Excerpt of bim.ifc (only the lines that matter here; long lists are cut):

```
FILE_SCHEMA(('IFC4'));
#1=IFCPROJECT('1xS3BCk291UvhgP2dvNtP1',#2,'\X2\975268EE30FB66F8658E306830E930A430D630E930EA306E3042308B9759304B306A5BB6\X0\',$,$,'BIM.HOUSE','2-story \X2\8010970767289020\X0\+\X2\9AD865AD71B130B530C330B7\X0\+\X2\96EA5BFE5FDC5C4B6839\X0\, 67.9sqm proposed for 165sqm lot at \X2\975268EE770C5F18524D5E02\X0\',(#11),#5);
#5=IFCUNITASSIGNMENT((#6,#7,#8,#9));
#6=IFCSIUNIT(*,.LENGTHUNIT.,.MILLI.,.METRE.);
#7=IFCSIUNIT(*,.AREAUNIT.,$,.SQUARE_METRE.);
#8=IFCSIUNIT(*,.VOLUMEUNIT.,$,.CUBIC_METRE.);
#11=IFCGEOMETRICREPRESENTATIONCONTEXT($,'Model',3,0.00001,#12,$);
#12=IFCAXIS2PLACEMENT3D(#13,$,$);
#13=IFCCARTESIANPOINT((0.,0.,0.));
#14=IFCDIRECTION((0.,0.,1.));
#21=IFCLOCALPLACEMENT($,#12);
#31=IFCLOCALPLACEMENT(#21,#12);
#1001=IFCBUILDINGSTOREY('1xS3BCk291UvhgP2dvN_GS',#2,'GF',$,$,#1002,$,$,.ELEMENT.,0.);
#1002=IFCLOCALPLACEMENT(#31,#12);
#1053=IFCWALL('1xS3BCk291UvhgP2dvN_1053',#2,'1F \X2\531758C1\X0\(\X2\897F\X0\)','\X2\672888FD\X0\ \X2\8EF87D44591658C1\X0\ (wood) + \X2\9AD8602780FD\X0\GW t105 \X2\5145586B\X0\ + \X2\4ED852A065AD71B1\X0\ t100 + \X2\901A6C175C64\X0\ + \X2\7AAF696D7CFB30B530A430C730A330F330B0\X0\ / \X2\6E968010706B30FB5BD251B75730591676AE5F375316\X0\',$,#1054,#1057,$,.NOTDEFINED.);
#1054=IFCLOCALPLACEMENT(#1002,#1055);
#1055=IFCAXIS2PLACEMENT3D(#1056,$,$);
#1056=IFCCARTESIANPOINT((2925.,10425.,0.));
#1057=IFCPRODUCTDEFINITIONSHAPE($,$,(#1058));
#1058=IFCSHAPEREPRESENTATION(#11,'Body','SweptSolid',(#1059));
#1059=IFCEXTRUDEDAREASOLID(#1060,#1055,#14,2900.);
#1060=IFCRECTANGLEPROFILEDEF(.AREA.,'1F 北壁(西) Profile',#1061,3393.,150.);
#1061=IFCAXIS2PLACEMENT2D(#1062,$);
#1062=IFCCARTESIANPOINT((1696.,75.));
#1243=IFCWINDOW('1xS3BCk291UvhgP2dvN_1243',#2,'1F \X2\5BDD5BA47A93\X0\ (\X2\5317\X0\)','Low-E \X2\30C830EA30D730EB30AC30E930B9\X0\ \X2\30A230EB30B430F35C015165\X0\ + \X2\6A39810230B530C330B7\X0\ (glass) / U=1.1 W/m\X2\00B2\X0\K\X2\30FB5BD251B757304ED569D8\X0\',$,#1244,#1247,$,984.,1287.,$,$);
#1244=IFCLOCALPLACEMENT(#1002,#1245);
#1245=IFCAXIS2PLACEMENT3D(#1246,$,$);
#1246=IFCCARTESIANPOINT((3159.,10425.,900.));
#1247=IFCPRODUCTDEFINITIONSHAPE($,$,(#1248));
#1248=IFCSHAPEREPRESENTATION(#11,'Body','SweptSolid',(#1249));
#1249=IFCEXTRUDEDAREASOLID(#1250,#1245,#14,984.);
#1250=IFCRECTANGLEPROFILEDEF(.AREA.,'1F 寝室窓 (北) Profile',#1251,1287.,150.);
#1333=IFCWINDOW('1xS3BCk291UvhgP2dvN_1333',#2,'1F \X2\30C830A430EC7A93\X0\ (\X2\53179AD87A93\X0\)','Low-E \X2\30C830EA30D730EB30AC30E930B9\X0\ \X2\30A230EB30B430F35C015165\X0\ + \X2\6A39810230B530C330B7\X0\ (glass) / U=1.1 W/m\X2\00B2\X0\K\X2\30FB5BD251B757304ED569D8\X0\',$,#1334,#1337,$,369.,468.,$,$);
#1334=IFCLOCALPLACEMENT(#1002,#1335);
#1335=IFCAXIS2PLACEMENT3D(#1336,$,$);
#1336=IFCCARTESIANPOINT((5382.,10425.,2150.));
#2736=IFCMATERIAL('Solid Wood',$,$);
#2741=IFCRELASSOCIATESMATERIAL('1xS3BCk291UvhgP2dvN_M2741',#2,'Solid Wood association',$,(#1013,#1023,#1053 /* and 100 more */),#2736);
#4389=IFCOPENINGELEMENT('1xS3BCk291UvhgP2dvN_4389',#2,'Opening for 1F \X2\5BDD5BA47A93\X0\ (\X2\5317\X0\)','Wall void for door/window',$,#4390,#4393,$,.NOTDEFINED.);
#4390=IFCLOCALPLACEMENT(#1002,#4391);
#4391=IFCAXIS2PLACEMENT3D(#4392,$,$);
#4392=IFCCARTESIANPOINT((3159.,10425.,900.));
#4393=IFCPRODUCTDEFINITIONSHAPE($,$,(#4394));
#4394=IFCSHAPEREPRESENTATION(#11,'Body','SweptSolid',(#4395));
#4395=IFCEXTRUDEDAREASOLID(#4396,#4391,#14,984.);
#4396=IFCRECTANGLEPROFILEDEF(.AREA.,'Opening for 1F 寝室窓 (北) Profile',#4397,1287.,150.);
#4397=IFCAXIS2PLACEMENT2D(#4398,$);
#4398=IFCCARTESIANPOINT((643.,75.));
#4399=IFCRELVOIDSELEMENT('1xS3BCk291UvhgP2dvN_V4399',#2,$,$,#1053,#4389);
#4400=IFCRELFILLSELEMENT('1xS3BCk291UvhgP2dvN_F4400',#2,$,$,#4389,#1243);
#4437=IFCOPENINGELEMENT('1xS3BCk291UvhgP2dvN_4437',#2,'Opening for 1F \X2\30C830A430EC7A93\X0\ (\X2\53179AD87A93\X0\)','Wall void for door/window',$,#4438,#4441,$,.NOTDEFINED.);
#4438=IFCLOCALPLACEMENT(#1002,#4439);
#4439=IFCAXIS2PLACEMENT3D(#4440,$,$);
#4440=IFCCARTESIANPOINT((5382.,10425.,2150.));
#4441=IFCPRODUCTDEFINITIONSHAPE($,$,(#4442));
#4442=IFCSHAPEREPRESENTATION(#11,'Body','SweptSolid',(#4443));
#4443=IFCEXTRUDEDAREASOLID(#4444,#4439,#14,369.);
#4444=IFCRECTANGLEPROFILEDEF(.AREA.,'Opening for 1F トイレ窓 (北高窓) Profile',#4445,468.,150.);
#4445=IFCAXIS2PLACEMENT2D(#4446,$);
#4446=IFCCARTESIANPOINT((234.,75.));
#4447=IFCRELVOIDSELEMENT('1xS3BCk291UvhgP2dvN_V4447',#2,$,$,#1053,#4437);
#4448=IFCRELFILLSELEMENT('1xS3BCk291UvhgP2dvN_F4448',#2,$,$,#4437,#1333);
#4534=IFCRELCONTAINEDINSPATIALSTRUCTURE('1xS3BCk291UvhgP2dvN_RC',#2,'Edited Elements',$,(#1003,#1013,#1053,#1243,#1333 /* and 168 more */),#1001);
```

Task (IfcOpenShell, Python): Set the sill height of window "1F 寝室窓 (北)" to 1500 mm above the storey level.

```python
import numpy as np
import ifcopenshell
import ifcopenshell.api.geometry
import ifcopenshell.geom
import ifcopenshell.util.element
import ifcopenshell.util.placement
import ifcopenshell.util.shape
import ifcopenshell.util.unit

model = ifcopenshell.open("bim.ifc")
unit_scale = ifcopenshell.util.unit.calculate_unit_scale(model)

window = model.by_id(1243)
opening = window.FillsVoids[0].RelatingOpeningElement
storey = ifcopenshell.util.element.get_container(window, ifc_class="IfcBuildingStorey")
level = ifcopenshell.util.placement.get_local_placement(storey.ObjectPlacement)[2, 3]

# The opening's origin need not be at the sill, so measure its lowest point.
shape = ifcopenshell.geom.create_shape(ifcopenshell.geom.settings(), opening)
bottom = ifcopenshell.util.shape.get_shape_bottom_elevation(shape, shape.geometry) / unit_scale
dz = level + 1.5 / unit_scale - bottom

shift = np.array([0.0, 0.0, dz])
# The window is not placed relative to its opening, so move both.
for product in (opening, window):
    matrix = ifcopenshell.util.placement.get_local_placement(product.ObjectPlacement)
    matrix[:3, 3] += shift
    ifcopenshell.api.geometry.edit_object_placement(model, product=product, matrix=matrix, is_si=False)

print(f"moved by {dz * unit_scale:+.3f} m")

model.write("bim_edited.ifc")
```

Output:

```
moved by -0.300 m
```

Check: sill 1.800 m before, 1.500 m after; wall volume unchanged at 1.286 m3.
